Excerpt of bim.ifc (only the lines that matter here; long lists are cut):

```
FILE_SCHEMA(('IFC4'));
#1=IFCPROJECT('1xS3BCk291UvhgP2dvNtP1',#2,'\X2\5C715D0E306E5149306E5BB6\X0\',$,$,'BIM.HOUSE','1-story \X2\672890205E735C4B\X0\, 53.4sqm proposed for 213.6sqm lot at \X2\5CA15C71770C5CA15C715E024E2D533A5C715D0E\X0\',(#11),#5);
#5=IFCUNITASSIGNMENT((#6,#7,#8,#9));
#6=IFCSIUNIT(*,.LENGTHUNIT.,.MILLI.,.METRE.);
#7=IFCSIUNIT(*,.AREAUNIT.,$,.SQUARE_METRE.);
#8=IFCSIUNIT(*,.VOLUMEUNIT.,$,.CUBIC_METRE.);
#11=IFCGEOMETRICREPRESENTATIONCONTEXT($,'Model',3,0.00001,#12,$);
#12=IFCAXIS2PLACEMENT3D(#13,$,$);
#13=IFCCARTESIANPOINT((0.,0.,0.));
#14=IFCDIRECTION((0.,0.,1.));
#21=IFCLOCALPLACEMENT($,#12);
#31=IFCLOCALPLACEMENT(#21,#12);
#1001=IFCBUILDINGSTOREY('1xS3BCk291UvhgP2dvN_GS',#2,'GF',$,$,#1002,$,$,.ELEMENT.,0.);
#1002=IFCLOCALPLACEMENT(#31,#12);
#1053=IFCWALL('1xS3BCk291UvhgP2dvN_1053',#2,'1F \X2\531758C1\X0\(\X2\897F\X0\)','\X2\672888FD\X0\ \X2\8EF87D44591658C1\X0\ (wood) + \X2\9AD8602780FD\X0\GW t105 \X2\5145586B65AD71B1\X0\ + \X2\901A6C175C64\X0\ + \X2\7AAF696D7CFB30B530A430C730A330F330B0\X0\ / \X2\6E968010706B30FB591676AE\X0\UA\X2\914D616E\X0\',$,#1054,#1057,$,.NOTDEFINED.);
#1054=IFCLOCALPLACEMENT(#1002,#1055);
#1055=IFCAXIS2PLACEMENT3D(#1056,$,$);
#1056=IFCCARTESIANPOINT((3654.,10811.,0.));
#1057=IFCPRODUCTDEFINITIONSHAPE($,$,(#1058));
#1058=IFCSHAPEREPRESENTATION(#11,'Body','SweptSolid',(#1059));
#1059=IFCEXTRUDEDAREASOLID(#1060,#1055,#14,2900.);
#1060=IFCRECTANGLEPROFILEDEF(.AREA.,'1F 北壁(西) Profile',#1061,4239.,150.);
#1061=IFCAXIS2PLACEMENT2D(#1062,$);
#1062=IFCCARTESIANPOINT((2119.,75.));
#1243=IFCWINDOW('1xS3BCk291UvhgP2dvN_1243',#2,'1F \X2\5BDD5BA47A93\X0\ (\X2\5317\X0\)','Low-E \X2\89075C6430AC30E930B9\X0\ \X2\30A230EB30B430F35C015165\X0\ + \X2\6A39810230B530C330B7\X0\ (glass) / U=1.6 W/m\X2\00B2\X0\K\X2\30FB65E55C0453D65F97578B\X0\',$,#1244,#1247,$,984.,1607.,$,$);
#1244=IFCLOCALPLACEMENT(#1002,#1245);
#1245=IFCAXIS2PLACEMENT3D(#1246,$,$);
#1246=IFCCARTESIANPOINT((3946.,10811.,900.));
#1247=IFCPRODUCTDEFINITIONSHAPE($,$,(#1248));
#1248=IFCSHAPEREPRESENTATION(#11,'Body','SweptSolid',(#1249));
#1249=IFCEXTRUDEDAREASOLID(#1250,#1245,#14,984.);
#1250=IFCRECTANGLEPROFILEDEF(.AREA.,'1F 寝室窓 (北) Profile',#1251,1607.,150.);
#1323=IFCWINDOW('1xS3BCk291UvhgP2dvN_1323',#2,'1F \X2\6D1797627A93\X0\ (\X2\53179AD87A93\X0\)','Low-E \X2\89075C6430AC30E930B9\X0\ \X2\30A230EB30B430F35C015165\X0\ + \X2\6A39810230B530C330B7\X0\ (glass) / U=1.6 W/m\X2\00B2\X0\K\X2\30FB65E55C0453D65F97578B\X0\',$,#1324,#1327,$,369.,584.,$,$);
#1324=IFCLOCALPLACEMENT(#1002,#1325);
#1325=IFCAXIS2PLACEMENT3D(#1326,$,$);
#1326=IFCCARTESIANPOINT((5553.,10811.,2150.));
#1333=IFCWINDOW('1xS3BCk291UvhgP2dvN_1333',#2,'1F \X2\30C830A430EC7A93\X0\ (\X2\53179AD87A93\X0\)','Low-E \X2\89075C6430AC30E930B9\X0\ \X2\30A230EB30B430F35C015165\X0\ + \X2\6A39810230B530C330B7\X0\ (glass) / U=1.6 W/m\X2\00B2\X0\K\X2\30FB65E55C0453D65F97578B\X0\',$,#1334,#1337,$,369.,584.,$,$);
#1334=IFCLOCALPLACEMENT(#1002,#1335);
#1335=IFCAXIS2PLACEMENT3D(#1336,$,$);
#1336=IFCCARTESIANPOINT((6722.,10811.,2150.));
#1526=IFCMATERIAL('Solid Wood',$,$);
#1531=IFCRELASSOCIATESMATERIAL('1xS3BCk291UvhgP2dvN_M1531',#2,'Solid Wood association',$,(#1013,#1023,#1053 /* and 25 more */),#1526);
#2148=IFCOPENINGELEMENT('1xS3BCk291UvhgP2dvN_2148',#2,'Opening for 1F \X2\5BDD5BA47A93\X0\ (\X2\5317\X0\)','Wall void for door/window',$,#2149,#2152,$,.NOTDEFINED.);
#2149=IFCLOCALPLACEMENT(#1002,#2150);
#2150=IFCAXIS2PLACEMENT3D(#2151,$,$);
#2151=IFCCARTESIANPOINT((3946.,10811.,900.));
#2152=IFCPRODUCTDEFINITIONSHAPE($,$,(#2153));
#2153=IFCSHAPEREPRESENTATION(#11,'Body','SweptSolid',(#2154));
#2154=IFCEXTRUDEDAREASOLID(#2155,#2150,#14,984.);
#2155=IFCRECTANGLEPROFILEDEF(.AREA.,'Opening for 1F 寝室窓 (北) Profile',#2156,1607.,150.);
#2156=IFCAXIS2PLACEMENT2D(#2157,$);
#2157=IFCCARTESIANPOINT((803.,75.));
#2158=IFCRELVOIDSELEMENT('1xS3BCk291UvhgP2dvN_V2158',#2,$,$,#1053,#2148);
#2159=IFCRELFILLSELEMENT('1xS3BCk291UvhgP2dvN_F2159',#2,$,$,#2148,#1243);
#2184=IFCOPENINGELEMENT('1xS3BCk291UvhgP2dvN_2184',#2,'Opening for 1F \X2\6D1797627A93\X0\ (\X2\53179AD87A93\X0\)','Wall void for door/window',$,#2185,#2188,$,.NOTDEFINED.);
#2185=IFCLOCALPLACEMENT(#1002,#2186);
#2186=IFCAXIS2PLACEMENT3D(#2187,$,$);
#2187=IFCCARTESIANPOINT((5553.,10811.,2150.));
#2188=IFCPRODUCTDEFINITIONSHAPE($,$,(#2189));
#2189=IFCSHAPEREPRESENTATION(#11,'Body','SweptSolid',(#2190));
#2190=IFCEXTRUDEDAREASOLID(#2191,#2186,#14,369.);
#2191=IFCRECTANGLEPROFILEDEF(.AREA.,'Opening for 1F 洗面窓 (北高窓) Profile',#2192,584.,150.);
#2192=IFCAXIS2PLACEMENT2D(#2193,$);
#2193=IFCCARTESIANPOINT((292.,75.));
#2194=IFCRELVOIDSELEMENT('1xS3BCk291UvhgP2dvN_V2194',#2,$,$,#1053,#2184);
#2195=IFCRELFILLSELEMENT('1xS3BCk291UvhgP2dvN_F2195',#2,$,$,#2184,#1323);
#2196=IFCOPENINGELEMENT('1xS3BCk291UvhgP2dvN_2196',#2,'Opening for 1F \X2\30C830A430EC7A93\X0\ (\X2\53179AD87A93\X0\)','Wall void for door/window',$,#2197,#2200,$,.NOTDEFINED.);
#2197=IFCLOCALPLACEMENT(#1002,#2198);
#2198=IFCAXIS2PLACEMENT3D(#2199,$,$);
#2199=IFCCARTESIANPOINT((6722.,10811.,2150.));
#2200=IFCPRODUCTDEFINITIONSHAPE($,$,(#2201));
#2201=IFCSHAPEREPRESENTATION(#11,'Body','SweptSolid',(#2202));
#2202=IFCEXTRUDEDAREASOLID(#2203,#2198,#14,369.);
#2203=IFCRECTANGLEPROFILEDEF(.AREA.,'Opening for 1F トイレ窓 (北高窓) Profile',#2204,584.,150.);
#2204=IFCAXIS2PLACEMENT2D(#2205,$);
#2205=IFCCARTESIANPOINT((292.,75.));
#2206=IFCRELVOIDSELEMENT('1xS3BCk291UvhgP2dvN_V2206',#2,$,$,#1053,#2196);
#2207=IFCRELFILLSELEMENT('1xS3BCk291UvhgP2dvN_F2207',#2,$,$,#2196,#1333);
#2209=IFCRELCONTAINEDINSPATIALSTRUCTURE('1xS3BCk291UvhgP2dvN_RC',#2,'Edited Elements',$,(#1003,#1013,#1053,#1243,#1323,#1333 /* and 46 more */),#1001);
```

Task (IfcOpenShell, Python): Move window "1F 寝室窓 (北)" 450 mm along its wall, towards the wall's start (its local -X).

```python
import ifcopenshell
import ifcopenshell.api.geometry
import ifcopenshell.util.placement
import ifcopenshell.util.unit

model = ifcopenshell.open("bim.ifc")
unit_scale = ifcopenshell.util.unit.calculate_unit_scale(model)

window = model.by_id(1243)
opening = window.FillsVoids[0].RelatingOpeningElement
wall = opening.VoidsElements[0].RelatingBuildingElement

wall_matrix = ifcopenshell.util.placement.get_local_placement(wall.ObjectPlacement)
shift = wall_matrix[:3, 0] * -0.45 / unit_scale
before = ifcopenshell.util.placement.get_local_placement(window.ObjectPlacement)[:3, 3].copy()

# The window is not placed relative to its opening, so move both.
for product in (opening, window):
    matrix = ifcopenshell.util.placement.get_local_placement(product.ObjectPlacement)
    matrix[:3, 3] += shift
    ifcopenshell.api.geometry.edit_object_placement(model, product=product, matrix=matrix, is_si=False)

after = ifcopenshell.util.placement.get_local_placement(window.ObjectPlacement)[:3, 3]
print("window moved by", (after - before).round(3) + 0.0)

model.write("bim_rev.ifc")
```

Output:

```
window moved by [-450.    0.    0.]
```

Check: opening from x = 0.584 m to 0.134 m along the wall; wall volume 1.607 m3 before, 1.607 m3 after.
